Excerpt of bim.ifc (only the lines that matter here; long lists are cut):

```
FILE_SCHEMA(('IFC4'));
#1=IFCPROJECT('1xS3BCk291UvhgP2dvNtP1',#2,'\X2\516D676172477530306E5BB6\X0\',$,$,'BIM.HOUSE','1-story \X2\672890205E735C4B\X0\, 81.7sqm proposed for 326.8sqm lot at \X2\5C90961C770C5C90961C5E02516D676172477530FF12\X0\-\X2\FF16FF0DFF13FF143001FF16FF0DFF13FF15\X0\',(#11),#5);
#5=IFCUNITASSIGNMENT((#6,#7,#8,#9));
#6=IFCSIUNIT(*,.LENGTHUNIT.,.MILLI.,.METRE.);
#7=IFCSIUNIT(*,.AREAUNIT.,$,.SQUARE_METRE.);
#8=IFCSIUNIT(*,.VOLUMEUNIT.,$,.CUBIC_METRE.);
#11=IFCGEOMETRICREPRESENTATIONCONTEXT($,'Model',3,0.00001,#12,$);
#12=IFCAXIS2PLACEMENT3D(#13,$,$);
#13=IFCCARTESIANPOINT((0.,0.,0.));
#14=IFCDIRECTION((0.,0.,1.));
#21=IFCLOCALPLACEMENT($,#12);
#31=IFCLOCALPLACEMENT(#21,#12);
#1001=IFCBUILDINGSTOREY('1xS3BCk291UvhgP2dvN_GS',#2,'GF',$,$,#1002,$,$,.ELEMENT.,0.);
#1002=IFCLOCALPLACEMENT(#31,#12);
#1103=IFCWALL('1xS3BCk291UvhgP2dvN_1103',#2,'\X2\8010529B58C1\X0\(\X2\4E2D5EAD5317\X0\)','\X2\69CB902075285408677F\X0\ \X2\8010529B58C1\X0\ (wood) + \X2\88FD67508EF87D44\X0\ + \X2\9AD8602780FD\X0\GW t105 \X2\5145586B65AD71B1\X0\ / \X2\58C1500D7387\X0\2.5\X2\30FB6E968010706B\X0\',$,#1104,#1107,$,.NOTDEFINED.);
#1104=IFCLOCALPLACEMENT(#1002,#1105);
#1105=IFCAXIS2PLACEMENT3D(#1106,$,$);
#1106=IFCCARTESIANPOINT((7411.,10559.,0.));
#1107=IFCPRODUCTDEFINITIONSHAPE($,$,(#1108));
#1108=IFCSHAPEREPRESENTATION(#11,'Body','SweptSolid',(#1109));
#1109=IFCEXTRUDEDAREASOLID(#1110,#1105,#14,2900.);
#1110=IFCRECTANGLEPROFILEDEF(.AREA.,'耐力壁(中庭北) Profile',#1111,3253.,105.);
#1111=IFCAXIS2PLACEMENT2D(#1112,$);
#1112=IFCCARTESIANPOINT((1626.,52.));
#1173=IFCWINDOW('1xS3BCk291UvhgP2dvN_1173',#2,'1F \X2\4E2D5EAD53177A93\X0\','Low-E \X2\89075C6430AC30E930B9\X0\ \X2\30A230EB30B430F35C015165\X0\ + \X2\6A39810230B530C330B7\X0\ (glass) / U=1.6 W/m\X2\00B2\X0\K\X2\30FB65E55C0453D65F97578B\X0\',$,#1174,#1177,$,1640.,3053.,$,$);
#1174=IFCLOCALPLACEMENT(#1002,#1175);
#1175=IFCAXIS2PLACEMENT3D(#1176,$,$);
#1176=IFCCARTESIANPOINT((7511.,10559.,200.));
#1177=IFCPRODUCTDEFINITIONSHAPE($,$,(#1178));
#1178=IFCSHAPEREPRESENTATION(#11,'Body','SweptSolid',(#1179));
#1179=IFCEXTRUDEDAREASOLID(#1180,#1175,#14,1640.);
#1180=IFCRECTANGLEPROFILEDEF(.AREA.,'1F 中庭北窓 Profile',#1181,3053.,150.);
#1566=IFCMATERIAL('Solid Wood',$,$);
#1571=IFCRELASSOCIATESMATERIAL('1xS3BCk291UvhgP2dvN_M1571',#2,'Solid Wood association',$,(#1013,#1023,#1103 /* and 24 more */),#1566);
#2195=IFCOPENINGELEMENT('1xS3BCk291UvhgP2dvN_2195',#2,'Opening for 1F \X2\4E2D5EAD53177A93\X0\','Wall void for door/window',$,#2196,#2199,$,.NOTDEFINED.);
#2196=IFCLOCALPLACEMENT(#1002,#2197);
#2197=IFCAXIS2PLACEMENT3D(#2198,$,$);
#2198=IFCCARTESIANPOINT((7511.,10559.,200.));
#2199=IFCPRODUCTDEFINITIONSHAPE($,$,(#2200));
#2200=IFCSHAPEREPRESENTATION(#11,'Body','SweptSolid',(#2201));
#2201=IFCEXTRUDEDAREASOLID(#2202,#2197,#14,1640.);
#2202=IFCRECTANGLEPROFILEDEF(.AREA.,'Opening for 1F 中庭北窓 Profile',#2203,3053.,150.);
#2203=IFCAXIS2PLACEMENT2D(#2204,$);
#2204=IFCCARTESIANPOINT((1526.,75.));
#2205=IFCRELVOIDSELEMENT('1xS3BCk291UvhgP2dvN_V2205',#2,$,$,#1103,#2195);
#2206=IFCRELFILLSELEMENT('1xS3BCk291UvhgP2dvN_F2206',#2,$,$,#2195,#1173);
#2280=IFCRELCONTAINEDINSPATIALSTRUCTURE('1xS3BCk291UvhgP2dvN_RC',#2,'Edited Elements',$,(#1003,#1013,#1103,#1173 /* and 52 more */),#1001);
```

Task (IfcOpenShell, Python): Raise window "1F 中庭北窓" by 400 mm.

```python
import numpy as np
import ifcopenshell
import ifcopenshell.api.geometry
import ifcopenshell.util.placement
import ifcopenshell.util.unit

model = ifcopenshell.open("bim.ifc")
unit_scale = ifcopenshell.util.unit.calculate_unit_scale(model)

window = model.by_id(1173)
opening = window.FillsVoids[0].RelatingOpeningElement
dz = 0.4 / unit_scale

shift = np.array([0.0, 0.0, dz])
# The window is not placed relative to its opening, so move both.
for product in (opening, window):
    matrix = ifcopenshell.util.placement.get_local_placement(product.ObjectPlacement)
    matrix[:3, 3] += shift
    ifcopenshell.api.geometry.edit_object_placement(model, product=product, matrix=matrix, is_si=False)

print(f"moved by {dz * unit_scale:+.3f} m")

model.write("bim_edited.ifc")
```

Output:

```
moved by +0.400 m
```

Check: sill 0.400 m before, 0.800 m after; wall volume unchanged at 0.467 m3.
